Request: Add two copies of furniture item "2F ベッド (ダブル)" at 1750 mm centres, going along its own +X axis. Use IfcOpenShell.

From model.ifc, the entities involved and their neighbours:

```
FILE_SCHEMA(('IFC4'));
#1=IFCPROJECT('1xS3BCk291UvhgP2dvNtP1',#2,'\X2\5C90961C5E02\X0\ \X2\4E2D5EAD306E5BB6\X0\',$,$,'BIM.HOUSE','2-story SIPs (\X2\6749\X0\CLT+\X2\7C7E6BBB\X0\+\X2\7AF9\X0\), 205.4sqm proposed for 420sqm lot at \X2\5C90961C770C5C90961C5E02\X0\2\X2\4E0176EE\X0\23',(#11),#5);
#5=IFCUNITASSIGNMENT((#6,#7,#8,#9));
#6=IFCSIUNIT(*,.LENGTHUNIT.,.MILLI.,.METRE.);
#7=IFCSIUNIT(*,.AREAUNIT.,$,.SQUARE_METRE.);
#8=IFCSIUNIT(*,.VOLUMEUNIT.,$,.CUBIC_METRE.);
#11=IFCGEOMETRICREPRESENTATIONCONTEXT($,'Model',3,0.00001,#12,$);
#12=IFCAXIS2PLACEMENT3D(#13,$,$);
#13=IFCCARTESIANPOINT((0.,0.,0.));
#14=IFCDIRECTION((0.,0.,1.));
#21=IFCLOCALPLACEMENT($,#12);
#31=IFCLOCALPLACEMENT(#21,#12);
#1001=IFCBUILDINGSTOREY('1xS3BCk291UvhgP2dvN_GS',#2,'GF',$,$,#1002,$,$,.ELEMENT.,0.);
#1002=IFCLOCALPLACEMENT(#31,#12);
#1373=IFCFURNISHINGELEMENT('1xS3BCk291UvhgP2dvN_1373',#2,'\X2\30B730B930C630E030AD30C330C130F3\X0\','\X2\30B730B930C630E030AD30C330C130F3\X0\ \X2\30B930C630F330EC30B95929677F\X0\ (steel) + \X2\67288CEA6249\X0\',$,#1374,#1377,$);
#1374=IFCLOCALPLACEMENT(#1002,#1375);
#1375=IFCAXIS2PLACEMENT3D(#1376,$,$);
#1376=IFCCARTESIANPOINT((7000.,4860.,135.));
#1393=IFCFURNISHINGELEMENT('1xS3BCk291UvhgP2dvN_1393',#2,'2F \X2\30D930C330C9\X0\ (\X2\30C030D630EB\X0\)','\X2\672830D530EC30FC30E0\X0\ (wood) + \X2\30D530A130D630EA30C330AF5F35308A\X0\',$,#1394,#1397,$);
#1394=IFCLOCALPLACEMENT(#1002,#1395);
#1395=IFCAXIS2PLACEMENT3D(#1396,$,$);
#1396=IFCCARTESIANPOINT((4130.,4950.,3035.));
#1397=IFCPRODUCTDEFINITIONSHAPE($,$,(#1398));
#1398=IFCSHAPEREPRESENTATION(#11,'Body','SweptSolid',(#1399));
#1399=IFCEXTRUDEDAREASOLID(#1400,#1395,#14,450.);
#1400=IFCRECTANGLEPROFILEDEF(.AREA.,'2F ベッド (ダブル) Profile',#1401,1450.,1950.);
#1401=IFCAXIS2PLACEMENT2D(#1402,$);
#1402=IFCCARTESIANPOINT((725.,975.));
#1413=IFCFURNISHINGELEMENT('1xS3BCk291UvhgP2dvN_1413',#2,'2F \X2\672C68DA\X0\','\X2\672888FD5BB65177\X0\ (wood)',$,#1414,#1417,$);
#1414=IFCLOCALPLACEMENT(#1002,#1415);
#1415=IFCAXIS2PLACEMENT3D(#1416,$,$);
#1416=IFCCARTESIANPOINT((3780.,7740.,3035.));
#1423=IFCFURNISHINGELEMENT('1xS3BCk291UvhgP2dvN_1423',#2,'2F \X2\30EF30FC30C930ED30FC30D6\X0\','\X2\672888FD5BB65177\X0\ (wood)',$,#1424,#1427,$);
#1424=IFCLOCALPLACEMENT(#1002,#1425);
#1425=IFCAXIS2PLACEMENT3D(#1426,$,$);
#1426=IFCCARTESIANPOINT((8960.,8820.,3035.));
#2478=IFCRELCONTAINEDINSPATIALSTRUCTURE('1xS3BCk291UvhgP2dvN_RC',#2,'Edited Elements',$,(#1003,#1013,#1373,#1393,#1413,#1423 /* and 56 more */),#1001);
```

```python
import ifcopenshell
import ifcopenshell.api.geometry
import ifcopenshell.api.root
import ifcopenshell.util.element
import ifcopenshell.util.placement

model = ifcopenshell.open("model.ifc")


def reuse_history(source, copy):
    """copy_class also copies each property set's owner history, people and application; keep the originals."""
    for rel in copy.IsDefinedBy:
        if rel.is_a("IfcRelDefinesByProperties") and (history := rel.RelatingPropertyDefinition.OwnerHistory):
            rel.RelatingPropertyDefinition.OwnerHistory = source.OwnerHistory
            ifcopenshell.util.element.remove_deep2(model, history)


source = model.by_guid("1xS3BCk291UvhgP2dvN_1393")
base = ifcopenshell.util.placement.get_local_placement(source.ObjectPlacement)
step = base[:3, 0] * 1750.0

for i in range(1, 3):
    copy = ifcopenshell.api.root.copy_class(model, product=source)
    copy.Representation = ifcopenshell.util.element.copy_deep(
        model, source.Representation, exclude=["IfcGeometricRepresentationContext", "IfcRepresentationMap"]
    )
    reuse_history(source, copy)
    matrix = base.copy()
    matrix[:3, 3] += i * step
    print("added at", matrix[:3, 3].round(3) + 0.0)
    ifcopenshell.api.geometry.edit_object_placement(model, product=copy, matrix=matrix, is_si=False)

model.write("model-out.ifc")
```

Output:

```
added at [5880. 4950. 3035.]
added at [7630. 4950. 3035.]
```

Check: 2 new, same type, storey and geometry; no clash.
